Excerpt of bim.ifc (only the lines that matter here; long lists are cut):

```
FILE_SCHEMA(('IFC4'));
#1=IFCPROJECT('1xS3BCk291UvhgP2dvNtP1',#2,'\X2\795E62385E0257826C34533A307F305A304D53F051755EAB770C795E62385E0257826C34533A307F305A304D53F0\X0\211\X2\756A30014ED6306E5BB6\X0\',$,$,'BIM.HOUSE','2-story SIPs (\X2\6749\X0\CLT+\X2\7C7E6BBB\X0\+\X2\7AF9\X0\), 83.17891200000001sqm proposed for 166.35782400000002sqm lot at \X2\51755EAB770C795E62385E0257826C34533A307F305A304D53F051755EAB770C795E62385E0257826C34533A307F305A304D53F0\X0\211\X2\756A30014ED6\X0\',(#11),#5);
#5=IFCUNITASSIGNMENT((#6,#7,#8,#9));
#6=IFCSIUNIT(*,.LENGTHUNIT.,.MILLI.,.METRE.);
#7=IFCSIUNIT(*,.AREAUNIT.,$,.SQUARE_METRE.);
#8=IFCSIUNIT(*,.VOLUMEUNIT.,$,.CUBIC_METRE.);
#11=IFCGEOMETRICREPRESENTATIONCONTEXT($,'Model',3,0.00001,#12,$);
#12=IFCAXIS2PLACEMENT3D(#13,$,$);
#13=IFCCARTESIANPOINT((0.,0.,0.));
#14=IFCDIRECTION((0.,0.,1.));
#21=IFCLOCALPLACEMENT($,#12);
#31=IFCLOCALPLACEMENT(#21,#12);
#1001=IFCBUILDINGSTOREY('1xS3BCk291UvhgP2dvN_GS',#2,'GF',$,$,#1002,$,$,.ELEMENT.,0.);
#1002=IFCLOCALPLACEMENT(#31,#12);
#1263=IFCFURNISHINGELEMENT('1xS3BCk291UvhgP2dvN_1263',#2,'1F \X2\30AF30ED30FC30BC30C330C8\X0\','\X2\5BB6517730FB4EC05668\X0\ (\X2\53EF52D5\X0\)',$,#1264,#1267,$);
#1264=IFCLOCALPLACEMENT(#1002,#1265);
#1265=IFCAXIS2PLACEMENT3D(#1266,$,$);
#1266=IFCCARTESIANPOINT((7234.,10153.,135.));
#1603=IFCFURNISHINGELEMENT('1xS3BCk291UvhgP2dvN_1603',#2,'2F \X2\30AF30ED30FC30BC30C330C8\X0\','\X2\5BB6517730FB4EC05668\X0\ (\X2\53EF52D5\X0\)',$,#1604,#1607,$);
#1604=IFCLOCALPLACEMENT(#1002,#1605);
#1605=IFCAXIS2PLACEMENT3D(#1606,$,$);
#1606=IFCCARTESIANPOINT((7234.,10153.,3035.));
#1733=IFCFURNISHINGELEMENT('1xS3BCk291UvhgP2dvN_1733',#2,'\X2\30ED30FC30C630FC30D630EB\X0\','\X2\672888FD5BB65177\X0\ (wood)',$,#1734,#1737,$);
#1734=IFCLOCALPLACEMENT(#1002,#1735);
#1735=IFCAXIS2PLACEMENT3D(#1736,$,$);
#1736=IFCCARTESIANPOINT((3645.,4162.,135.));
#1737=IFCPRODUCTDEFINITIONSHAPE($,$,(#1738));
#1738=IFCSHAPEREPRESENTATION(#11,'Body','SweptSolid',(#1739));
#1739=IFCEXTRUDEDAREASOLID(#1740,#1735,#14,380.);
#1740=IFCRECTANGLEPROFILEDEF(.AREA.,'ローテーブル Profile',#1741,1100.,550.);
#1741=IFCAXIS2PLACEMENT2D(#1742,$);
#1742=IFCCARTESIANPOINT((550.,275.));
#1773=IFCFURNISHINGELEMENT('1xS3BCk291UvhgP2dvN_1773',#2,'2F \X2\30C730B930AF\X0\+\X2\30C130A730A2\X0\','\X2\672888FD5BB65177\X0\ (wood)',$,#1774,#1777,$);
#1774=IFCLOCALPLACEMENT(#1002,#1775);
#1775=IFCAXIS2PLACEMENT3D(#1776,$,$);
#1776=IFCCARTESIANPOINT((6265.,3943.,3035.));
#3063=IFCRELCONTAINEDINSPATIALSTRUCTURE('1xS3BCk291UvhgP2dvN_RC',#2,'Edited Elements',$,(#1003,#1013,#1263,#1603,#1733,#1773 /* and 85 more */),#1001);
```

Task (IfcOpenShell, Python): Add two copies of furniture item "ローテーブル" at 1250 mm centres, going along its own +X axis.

```python
import ifcopenshell
import ifcopenshell.api.geometry
import ifcopenshell.api.root
import ifcopenshell.util.element
import ifcopenshell.util.placement

model = ifcopenshell.open("bim.ifc")


def reuse_history(source, copy):
    """copy_class also copies each property set's owner history, people and application; keep the originals."""
    for rel in copy.IsDefinedBy:
        if rel.is_a("IfcRelDefinesByProperties") and (history := rel.RelatingPropertyDefinition.OwnerHistory):
            rel.RelatingPropertyDefinition.OwnerHistory = source.OwnerHistory
            ifcopenshell.util.element.remove_deep2(model, history)


source = model.by_id(1733)
base = ifcopenshell.util.placement.get_local_placement(source.ObjectPlacement)
step = base[:3, 0] * 1250.0

for i in range(1, 3):
    copy = ifcopenshell.api.root.copy_class(model, product=source)
    copy.Representation = ifcopenshell.util.element.copy_deep(
        model, source.Representation, exclude=["IfcGeometricRepresentationContext", "IfcRepresentationMap"]
    )
    reuse_history(source, copy)
    matrix = base.copy()
    matrix[:3, 3] += i * step
    print("added at", matrix[:3, 3].round(3) + 0.0)
    ifcopenshell.api.geometry.edit_object_placement(model, product=copy, matrix=matrix, is_si=False)

model.write("bim_rev.ifc")
```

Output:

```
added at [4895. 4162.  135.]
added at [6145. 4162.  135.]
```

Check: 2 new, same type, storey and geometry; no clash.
